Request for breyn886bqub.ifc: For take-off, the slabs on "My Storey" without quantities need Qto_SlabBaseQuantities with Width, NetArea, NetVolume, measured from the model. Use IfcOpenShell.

First a look at what the model holds.

```python
import ifcopenshell
import ifcopenshell.util.element
import ifcopenshell.util.unit

model = ifcopenshell.open("breyn886bqub.ifc")
print(model.schema)
for unit_type in ("LENGTHUNIT", "AREAUNIT", "VOLUMEUNIT"):
    print(unit_type, ifcopenshell.util.unit.calculate_unit_scale(model, unit_type))
storey = next(s for s in model.by_type("IfcBuildingStorey") if s.Name == "My Storey")
slabs = [e for e in ifcopenshell.util.element.get_decomposition(storey) if e.is_a("IfcSlab")]
for e in sorted(slabs, key=lambda e: e.id()):
    print(e.id(), e.is_a(), e.Name, list(ifcopenshell.util.element.get_psets(e, qtos_only=True)), sep=" | ")
```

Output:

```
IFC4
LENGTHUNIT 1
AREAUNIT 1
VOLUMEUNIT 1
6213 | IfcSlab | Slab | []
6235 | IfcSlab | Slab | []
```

```python
import ifcopenshell
import ifcopenshell.api.pset
import ifcopenshell.geom
import ifcopenshell.util.element
import ifcopenshell.util.shape
import ifcopenshell.util.unit

model = ifcopenshell.open("breyn886bqub.ifc")
unit_scale = ifcopenshell.util.unit.calculate_unit_scale(model)
area_scale = ifcopenshell.util.unit.calculate_unit_scale(model, "AREAUNIT")
volume_scale = ifcopenshell.util.unit.calculate_unit_scale(model, "VOLUMEUNIT")
settings = ifcopenshell.geom.settings()

storey = next(s for s in model.by_type("IfcBuildingStorey") if s.Name == "My Storey")
slabs = [e for e in ifcopenshell.util.element.get_decomposition(storey) if e.is_a("IfcSlab")]

for e in sorted(slabs, key=lambda e: e.id()):
    if ifcopenshell.util.element.get_psets(e, qtos_only=True, should_inherit=False):
        continue
    # Geometry comes back in metres, in the element's own axes.
    shape = ifcopenshell.geom.create_shape(settings, e)
    values = {
        "Width": ifcopenshell.util.shape.get_z(shape.geometry) / unit_scale,
        "NetArea": ifcopenshell.util.shape.get_footprint_area(shape.geometry) / area_scale,
        "NetVolume": ifcopenshell.util.shape.get_volume(shape.geometry) / volume_scale,
    }
    qto = ifcopenshell.api.pset.add_qto(model, product=e, name="Qto_SlabBaseQuantities")
    ifcopenshell.api.pset.edit_qto(model, qto=qto, properties=values)
    print(e.id(), {k: round(v, 3) for k, v in values.items()})

model.write("breyn886bqub_rev.ifc")
```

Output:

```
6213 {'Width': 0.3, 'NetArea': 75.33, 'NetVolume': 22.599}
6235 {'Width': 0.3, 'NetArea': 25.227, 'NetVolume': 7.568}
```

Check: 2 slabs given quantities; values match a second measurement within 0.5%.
